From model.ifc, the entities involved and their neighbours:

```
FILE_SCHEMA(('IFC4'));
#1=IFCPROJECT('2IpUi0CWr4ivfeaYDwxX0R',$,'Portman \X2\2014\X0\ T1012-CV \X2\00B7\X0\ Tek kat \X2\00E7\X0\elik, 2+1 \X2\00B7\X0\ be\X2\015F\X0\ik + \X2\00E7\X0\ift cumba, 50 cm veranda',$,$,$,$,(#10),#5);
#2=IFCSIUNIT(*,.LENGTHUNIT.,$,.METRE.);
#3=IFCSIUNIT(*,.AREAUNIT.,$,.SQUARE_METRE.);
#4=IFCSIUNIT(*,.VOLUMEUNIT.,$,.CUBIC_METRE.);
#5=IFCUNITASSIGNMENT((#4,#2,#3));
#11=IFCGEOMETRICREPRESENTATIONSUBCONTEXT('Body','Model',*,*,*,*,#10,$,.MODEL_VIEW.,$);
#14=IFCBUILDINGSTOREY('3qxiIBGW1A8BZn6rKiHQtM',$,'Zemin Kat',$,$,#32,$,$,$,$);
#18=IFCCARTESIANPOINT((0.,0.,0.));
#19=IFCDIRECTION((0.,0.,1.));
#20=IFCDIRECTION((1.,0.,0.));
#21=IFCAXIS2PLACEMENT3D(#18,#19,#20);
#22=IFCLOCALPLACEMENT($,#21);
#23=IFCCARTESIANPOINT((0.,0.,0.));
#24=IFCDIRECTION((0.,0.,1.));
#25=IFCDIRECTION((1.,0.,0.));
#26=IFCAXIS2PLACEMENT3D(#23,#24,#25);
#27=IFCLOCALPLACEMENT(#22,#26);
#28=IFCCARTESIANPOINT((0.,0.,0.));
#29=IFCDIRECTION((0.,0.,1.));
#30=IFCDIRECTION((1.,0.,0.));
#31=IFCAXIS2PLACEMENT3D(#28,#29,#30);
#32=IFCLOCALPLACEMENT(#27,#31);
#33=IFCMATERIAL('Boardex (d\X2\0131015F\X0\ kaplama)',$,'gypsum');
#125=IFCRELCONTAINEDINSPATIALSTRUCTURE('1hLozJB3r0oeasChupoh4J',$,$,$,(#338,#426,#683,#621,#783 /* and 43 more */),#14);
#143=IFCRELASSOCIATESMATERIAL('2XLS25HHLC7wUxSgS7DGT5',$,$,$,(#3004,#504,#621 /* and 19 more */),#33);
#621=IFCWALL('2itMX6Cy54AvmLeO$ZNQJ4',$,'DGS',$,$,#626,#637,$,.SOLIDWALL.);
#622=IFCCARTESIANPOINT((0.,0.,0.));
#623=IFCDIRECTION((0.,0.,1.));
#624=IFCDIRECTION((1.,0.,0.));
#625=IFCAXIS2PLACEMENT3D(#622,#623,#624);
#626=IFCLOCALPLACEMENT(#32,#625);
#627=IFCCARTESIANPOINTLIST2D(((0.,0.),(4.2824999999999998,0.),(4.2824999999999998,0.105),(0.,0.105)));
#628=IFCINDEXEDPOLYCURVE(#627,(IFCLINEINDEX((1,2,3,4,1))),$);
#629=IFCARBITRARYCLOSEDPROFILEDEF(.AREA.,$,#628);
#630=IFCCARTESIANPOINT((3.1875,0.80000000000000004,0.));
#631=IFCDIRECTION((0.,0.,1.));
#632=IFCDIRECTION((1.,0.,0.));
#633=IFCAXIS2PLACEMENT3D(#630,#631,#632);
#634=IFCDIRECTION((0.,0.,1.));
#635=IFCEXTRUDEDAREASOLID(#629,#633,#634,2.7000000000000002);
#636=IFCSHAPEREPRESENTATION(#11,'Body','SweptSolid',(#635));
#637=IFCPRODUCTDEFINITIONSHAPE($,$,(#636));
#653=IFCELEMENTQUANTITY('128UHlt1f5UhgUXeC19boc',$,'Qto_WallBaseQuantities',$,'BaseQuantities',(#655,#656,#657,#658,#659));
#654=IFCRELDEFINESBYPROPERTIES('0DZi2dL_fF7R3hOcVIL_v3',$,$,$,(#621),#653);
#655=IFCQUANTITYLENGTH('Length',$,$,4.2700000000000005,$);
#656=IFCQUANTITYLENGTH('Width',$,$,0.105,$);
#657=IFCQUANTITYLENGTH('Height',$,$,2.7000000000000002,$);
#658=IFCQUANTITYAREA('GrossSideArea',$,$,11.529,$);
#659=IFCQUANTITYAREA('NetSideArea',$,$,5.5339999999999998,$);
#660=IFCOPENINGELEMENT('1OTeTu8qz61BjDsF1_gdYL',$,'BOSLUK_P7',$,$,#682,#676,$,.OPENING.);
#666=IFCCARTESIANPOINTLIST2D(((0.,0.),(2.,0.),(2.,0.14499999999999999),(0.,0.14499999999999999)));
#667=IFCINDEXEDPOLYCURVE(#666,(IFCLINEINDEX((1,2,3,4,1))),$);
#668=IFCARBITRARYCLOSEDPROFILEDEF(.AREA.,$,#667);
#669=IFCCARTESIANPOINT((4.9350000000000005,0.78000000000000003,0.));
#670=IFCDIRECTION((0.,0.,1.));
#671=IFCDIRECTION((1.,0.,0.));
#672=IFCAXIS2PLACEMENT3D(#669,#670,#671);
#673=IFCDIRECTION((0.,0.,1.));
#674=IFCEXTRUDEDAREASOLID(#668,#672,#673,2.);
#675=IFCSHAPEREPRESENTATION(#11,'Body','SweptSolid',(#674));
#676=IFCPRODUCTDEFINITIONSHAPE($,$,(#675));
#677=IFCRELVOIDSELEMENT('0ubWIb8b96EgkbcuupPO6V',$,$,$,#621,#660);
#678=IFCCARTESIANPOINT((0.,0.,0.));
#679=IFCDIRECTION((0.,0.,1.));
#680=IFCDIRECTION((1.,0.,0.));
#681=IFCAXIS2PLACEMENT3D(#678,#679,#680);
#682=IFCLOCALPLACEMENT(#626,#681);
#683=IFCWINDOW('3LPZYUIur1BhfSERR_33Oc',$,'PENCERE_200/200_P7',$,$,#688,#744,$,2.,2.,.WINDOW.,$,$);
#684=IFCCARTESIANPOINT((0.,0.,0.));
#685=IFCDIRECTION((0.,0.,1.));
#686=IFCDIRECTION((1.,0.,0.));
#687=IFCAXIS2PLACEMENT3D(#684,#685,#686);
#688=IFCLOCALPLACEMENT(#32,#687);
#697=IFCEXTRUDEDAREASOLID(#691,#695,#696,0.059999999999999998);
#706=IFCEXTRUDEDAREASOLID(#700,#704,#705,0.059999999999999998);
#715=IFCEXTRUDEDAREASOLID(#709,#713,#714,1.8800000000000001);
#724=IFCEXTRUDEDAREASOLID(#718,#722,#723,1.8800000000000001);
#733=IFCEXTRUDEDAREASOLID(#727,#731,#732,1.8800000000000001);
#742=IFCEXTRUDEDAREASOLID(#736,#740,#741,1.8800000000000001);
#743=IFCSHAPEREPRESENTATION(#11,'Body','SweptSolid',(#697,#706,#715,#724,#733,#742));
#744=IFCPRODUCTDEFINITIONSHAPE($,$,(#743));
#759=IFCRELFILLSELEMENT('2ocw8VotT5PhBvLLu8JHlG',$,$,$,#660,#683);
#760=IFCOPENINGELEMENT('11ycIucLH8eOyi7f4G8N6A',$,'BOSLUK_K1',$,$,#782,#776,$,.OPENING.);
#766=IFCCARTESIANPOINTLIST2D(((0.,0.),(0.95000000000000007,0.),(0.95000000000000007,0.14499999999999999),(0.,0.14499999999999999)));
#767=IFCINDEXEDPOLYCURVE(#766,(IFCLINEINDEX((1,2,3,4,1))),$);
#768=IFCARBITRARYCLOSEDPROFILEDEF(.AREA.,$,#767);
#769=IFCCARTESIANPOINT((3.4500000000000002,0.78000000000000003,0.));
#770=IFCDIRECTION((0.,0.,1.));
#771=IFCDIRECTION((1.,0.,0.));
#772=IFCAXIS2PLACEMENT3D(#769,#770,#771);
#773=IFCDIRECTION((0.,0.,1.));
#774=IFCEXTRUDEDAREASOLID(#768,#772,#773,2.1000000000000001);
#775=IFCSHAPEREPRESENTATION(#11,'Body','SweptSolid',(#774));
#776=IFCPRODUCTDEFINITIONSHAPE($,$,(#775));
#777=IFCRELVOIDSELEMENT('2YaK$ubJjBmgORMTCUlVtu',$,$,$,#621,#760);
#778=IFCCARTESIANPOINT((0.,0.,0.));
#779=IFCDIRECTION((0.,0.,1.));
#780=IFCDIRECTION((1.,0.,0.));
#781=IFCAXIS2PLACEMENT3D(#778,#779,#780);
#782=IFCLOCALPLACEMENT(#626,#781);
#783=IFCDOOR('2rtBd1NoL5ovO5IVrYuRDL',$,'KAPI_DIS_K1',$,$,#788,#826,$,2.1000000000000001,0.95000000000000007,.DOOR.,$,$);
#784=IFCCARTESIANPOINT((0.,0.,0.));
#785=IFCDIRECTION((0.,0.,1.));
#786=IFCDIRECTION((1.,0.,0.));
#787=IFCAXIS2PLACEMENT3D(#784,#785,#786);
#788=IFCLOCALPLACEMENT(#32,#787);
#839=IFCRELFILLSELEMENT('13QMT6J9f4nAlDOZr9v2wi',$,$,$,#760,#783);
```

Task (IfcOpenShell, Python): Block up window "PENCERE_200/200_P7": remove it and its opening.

```python
import ifcopenshell
import ifcopenshell.api.feature
import ifcopenshell.api.pset
import ifcopenshell.api.root
import ifcopenshell.geom
import ifcopenshell.util.element
import ifcopenshell.util.shape
import ifcopenshell.util.unit

model = ifcopenshell.open("model.ifc")
area_scale = ifcopenshell.util.unit.calculate_unit_scale(model, "AREAUNIT")
settings = ifcopenshell.geom.settings()


def volume(element):
    """Net volume in cubic metres, openings subtracted."""
    shape = ifcopenshell.geom.create_shape(settings, element)
    return ifcopenshell.util.shape.get_volume(shape.geometry)


window = model.by_id(683)
opening = window.FillsVoids[0].RelatingOpeningElement
wall = opening.VoidsElements[0].RelatingBuildingElement
before = volume(wall)

ifcopenshell.api.root.remove_product(model, product=window)
ifcopenshell.api.feature.remove_feature(model, feature=opening)

after = volume(wall)
thickness = 0.105  # wall thickness in metres

# Update the wall's stored quantities.
qto = model.by_id(ifcopenshell.util.element.get_pset(wall, "Qto_WallBaseQuantities", should_inherit=False)["id"])
ifcopenshell.api.pset.edit_qto(model, qto=qto, properties={"NetSideArea": after / thickness / area_scale})

print(f"wall volume {before:.3f} -> {after:.3f} m3")

model.write("model_rev.ifc")
```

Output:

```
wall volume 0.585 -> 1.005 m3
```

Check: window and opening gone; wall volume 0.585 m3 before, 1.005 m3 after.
